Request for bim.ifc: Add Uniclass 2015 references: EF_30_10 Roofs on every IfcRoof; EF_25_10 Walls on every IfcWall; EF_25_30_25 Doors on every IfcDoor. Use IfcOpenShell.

First a look at what the model holds.

```python
import ifcopenshell

model = ifcopenshell.open("bim.ifc")
print(model.schema)
print("classifications:", [c.Name for c in model.by_type("IfcClassification")])
for ifc_class in ("IfcDoor", "IfcRoof", "IfcStair", "IfcWall", "IfcWindow"):
    print(ifc_class, len(model.by_type(ifc_class)))
```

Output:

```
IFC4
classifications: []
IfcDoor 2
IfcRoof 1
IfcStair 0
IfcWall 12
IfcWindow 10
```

```python
import ifcopenshell
import ifcopenshell.api.classification

model = ifcopenshell.open("bim.ifc")

system = ifcopenshell.api.classification.add_classification(model, classification="Uniclass 2015")

codes = {
    "IfcRoof": ("EF_30_10", "Roofs"),
    "IfcWall": ("EF_25_10", "Walls"),
    "IfcDoor": ("EF_25_30_25", "Doors"),
}
for ifc_class, (code, name) in codes.items():
    products = model.by_type(ifc_class)
    ifcopenshell.api.classification.add_reference(
        model, products=products, classification=system, identification=code, name=name
    )
    print(code, len(products))

model.write("bim_rev.ifc")
```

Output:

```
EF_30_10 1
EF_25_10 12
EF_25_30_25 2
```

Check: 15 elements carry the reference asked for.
